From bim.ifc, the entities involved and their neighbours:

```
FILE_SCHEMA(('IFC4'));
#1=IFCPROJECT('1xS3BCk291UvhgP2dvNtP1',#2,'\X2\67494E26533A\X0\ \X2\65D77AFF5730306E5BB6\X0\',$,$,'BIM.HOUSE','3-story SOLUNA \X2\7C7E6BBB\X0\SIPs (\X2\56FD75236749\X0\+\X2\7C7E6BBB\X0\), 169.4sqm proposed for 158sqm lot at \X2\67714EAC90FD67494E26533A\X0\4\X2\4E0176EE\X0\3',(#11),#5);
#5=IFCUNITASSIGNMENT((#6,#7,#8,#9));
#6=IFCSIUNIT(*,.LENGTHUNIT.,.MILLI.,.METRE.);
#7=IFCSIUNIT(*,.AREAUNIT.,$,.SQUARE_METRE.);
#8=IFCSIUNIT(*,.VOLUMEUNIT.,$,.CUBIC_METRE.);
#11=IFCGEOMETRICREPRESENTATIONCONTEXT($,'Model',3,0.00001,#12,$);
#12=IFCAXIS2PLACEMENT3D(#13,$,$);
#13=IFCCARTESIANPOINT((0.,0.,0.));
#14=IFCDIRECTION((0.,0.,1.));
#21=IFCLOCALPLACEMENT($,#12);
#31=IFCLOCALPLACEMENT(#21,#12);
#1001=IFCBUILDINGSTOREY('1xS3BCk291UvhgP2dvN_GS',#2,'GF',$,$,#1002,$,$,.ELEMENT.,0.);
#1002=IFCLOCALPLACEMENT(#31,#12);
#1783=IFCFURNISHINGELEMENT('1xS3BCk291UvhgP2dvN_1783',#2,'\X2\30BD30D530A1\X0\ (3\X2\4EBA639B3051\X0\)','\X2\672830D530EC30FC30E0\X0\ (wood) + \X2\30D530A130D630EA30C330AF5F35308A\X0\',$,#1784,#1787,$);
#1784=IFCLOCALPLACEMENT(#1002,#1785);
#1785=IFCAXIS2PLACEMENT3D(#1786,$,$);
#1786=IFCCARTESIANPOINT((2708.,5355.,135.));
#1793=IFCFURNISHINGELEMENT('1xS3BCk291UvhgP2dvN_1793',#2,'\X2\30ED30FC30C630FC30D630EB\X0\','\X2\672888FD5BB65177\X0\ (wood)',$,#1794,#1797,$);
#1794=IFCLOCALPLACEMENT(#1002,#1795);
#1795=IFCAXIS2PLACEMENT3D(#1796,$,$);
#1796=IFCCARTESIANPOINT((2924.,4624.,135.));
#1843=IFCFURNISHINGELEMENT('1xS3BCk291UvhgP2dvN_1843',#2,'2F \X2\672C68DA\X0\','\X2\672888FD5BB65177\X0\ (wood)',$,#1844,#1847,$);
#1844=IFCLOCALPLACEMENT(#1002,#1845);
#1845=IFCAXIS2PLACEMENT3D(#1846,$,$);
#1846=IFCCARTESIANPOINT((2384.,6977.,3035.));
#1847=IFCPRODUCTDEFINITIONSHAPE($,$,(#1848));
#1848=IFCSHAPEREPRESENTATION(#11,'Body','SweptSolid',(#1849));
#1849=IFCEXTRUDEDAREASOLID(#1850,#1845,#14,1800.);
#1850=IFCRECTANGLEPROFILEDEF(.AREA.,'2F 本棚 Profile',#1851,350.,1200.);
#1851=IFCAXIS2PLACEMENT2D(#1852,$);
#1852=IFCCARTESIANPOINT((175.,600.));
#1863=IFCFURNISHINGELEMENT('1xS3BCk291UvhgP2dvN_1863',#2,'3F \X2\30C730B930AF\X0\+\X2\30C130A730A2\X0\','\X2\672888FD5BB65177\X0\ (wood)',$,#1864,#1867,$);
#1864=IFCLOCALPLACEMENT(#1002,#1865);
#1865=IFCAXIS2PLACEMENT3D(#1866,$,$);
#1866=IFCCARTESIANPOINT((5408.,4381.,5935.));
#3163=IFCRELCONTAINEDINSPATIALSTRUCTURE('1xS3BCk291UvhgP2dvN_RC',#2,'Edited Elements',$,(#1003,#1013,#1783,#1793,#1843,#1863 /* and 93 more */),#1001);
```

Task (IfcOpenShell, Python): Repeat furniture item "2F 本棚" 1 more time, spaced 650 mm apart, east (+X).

```python
import numpy as np
import ifcopenshell
import ifcopenshell.api.geometry
import ifcopenshell.api.root
import ifcopenshell.util.element
import ifcopenshell.util.placement
import ifcopenshell.util.unit

model = ifcopenshell.open("bim.ifc")
unit_scale = ifcopenshell.util.unit.calculate_unit_scale(model)


def reuse_history(source, copy):
    """copy_class also copies each property set's owner history, people and application; keep the originals."""
    for rel in copy.IsDefinedBy:
        if rel.is_a("IfcRelDefinesByProperties") and (history := rel.RelatingPropertyDefinition.OwnerHistory):
            rel.RelatingPropertyDefinition.OwnerHistory = source.OwnerHistory
            ifcopenshell.util.element.remove_deep2(model, history)


source = model.by_id(1843)
base = ifcopenshell.util.placement.get_local_placement(source.ObjectPlacement)
step = np.array([1.0, 0.0, 0.0]) * 0.65 / unit_scale

for i in range(1, 2):
    copy = ifcopenshell.api.root.copy_class(model, product=source)
    copy.Representation = ifcopenshell.util.element.copy_deep(
        model, source.Representation, exclude=["IfcGeometricRepresentationContext", "IfcRepresentationMap"]
    )
    reuse_history(source, copy)
    matrix = base.copy()
    matrix[:3, 3] += i * step
    print("added at", matrix[:3, 3].round(3) + 0.0)
    ifcopenshell.api.geometry.edit_object_placement(model, product=copy, matrix=matrix, is_si=False)

model.write("bim_rev.ifc")
```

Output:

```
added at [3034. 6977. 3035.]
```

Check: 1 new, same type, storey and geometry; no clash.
